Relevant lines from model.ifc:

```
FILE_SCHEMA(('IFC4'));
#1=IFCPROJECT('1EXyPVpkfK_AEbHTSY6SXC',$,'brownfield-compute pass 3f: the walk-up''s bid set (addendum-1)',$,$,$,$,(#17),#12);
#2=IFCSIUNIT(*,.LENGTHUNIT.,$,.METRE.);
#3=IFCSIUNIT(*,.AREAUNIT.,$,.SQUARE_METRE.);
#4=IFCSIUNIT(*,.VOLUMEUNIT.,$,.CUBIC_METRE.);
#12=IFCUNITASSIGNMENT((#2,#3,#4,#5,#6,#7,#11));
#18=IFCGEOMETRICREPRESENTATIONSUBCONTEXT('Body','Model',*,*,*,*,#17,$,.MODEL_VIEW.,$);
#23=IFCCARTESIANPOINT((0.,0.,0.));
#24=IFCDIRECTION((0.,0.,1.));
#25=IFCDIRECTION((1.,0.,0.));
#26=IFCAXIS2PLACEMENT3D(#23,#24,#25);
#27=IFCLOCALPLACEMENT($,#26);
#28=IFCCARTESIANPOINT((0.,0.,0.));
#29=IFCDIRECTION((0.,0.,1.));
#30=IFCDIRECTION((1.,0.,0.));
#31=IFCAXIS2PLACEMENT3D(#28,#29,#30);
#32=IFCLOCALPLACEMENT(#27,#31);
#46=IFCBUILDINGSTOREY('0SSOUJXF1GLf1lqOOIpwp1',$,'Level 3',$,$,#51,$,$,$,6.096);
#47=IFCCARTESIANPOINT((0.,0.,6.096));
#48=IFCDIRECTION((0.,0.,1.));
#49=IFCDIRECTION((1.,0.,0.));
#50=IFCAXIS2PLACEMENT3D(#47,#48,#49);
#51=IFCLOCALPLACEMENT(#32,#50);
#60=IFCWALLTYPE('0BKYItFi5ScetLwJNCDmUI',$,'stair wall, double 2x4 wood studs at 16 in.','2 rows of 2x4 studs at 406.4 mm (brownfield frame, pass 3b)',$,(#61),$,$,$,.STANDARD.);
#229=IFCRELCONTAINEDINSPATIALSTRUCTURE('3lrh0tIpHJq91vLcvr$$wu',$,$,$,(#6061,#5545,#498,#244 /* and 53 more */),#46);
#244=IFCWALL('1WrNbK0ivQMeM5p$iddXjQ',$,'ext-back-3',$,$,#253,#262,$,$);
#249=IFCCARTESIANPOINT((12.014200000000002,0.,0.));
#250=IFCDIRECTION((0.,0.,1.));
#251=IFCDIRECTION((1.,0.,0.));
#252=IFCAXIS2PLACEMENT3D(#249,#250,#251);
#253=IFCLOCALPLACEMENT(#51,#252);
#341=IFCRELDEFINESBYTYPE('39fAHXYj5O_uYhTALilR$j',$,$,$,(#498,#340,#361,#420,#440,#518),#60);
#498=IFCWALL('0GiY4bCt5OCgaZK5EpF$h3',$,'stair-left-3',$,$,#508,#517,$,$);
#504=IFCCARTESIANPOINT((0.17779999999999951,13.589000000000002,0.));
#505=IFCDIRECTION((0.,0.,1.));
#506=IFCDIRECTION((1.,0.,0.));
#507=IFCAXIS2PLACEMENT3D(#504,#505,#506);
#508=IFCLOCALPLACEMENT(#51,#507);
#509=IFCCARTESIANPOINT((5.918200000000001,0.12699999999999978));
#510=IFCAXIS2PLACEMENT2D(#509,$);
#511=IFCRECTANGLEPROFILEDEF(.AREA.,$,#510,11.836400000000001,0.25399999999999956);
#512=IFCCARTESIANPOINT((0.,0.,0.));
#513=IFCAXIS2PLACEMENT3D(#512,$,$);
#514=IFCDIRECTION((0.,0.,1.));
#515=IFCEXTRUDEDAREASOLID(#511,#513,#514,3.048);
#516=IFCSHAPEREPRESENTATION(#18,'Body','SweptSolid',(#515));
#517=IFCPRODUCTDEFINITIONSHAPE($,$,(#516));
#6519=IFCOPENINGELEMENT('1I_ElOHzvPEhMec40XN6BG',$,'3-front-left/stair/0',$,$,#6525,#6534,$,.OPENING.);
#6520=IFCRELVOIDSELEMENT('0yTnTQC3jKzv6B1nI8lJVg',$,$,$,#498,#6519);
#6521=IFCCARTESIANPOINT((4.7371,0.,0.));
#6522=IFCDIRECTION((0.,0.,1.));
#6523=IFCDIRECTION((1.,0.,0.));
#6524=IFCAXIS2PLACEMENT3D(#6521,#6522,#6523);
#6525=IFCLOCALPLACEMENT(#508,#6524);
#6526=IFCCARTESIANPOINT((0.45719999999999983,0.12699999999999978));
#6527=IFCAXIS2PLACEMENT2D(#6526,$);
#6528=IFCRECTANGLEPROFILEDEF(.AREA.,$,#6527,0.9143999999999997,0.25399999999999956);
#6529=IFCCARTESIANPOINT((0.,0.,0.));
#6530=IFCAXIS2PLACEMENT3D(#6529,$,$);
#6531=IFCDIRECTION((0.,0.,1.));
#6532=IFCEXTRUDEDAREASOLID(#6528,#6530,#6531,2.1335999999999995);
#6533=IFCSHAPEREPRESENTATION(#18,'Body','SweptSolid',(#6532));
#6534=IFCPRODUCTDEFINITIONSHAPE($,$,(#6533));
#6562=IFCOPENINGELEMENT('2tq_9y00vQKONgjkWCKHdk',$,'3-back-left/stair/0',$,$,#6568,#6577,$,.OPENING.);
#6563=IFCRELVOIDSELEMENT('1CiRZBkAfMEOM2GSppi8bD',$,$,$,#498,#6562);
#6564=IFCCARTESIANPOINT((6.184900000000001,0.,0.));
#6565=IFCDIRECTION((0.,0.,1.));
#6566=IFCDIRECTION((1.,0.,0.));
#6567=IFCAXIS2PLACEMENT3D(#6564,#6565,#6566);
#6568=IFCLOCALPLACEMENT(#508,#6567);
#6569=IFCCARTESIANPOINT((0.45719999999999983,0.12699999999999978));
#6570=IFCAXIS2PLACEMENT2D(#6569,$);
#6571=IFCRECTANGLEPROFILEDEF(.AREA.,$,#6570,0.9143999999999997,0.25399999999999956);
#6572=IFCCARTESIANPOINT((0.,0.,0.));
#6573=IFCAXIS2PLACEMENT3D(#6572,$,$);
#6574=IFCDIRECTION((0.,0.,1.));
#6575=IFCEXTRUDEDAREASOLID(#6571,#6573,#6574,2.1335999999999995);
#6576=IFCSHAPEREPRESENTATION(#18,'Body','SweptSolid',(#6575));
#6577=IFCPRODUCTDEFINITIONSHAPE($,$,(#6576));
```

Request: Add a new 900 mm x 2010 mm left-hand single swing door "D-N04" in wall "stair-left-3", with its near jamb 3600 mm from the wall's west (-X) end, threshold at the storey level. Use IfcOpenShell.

```python
import numpy as np
import ifcopenshell
import ifcopenshell.api.feature
import ifcopenshell.api.geometry
import ifcopenshell.api.root
import ifcopenshell.api.spatial
import ifcopenshell.geom
import ifcopenshell.util.element
import ifcopenshell.util.placement
import ifcopenshell.util.representation
import ifcopenshell.util.shape
import ifcopenshell.util.unit

model = ifcopenshell.open("model.ifc")
unit_scale = ifcopenshell.util.unit.calculate_unit_scale(model)
settings = ifcopenshell.geom.settings()


def volume(element):
    """Net volume in cubic metres, openings subtracted."""
    shape = ifcopenshell.geom.create_shape(settings, element)
    return ifcopenshell.util.shape.get_volume(shape.geometry)


wall = model.by_id(498)
storey = ifcopenshell.util.element.get_container(wall, ifc_class="IfcBuildingStorey")
context = ifcopenshell.util.representation.get_context(model, "Model", "Body", "MODEL_VIEW")
before = volume(wall)

width, height, from_end, sill = 0.9, 2.01, 3.6, 0.0  # metres

# The wall runs along its own X axis, and the end named is its -X end.
wall_shape = ifcopenshell.geom.create_shape(settings, wall)
x, y, z = ifcopenshell.util.shape.get_vertices(wall_shape.geometry).T
start = x.min() + from_end
face, thickness = float(y.min()), float(y.max() - y.min())
wall_matrix = ifcopenshell.util.placement.get_local_placement(wall.ObjectPlacement)
level = ifcopenshell.util.placement.get_local_placement(storey.ObjectPlacement)[2, 3]


def in_wall(x, y):
    """Placement at x, y metres in the wall's axes, at sill height."""
    matrix = wall_matrix.copy()
    matrix[:, 3] = wall_matrix @ np.array([x / unit_scale, y / unit_scale, 0.0, 1.0])
    matrix[2, 3] = level + sill / unit_scale
    return matrix


# Opening: a box that overshoots both wall faces by 50 mm.
opening = ifcopenshell.api.root.create_entity(model, ifc_class="IfcOpeningElement", predefined_type="OPENING")
box = ifcopenshell.api.geometry.add_wall_representation(
    model, context=context, length=width, height=height, thickness=thickness + 0.1
)
ifcopenshell.api.geometry.assign_representation(model, product=opening, representation=box)
ifcopenshell.api.geometry.edit_object_placement(model, product=opening, matrix=in_wall(start, face - 0.05), is_si=False)
ifcopenshell.api.feature.add_feature(model, feature=opening, element=wall)

door = ifcopenshell.api.root.create_entity(model, ifc_class="IfcDoor", name="D-N04", predefined_type="DOOR")
door.OverallWidth, door.OverallHeight = width / unit_scale, height / unit_scale
door.OperationType = "SINGLE_SWING_LEFT"
body = ifcopenshell.api.geometry.add_door_representation(
    model,
    context=context,
    overall_width=door.OverallWidth,
    overall_height=door.OverallHeight,
    operation_type="SINGLE_SWING_LEFT",
    lining_properties={"LiningDepth": thickness / unit_scale, "ThresholdDepth": thickness / unit_scale},
)
ifcopenshell.api.geometry.assign_representation(model, product=door, representation=body)
ifcopenshell.api.spatial.assign_container(model, products=[door], relating_structure=storey)
ifcopenshell.api.feature.add_filling(model, opening=opening, element=door)

# The lining spans the wall, so the door starts at the wall face.
ifcopenshell.api.geometry.edit_object_placement(model, product=door, matrix=in_wall(start, face), is_si=False)

after = volume(wall)

print(f"wall volume {before:.3f} -> {after:.3f} m3")

model.write("model_updated.ifc")
```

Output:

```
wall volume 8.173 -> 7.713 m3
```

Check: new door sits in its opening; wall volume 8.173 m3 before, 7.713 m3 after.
